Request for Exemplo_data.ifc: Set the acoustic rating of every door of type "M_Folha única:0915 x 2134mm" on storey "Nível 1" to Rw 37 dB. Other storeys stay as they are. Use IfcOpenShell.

First a look at what the model holds.

```python
import ifcopenshell
import ifcopenshell.util.element

model = ifcopenshell.open("Exemplo_data.ifc")
print(model.schema)
storey = next(s for s in model.by_type("IfcBuildingStorey") if s.Name == "Nível 1")
doors = [e for e in ifcopenshell.util.element.get_decomposition(storey) if e.is_a("IfcDoor")]
seen = {}
for e in doors:
    element_type = ifcopenshell.util.element.get_type(e)
    key = (element_type.Name if element_type != e and element_type else None, ifcopenshell.util.element.get_pset(e, "Pset_DoorCommon", "AcousticRating"))
    seen[key] = seen.get(key, 0) + 1
for (name, value), count in sorted(seen.items(), key=str):
    print(count, "x", name, "|", value)
```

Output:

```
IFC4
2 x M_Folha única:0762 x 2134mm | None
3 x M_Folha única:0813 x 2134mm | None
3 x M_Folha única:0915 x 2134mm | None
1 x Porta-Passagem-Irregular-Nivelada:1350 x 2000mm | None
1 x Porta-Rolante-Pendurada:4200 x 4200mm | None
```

```python
import ifcopenshell
import ifcopenshell.api.pset
import ifcopenshell.util.element

model = ifcopenshell.open("Exemplo_data.ifc")

storey = next(s for s in model.by_type("IfcBuildingStorey") if s.Name == "Nível 1")
doors = [e for e in ifcopenshell.util.element.get_decomposition(storey) if e.is_a("IfcDoor")]

count = 0
for e in doors:
    element_type = ifcopenshell.util.element.get_type(e)
    if element_type in (None, e) or element_type.Name != "M_Folha única:0915 x 2134mm":
        continue
    # add_pset returns the element's existing set when there is one.
    pset = ifcopenshell.api.pset.add_pset(model, product=e, name="Pset_DoorCommon")
    ifcopenshell.api.pset.edit_pset(model, pset=pset, properties={"AcousticRating": "Rw 37 dB"})
    count += 1

print(count, "doors updated")

model.write("Exemplo_data_rev.ifc")
```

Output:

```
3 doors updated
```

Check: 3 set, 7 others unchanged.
